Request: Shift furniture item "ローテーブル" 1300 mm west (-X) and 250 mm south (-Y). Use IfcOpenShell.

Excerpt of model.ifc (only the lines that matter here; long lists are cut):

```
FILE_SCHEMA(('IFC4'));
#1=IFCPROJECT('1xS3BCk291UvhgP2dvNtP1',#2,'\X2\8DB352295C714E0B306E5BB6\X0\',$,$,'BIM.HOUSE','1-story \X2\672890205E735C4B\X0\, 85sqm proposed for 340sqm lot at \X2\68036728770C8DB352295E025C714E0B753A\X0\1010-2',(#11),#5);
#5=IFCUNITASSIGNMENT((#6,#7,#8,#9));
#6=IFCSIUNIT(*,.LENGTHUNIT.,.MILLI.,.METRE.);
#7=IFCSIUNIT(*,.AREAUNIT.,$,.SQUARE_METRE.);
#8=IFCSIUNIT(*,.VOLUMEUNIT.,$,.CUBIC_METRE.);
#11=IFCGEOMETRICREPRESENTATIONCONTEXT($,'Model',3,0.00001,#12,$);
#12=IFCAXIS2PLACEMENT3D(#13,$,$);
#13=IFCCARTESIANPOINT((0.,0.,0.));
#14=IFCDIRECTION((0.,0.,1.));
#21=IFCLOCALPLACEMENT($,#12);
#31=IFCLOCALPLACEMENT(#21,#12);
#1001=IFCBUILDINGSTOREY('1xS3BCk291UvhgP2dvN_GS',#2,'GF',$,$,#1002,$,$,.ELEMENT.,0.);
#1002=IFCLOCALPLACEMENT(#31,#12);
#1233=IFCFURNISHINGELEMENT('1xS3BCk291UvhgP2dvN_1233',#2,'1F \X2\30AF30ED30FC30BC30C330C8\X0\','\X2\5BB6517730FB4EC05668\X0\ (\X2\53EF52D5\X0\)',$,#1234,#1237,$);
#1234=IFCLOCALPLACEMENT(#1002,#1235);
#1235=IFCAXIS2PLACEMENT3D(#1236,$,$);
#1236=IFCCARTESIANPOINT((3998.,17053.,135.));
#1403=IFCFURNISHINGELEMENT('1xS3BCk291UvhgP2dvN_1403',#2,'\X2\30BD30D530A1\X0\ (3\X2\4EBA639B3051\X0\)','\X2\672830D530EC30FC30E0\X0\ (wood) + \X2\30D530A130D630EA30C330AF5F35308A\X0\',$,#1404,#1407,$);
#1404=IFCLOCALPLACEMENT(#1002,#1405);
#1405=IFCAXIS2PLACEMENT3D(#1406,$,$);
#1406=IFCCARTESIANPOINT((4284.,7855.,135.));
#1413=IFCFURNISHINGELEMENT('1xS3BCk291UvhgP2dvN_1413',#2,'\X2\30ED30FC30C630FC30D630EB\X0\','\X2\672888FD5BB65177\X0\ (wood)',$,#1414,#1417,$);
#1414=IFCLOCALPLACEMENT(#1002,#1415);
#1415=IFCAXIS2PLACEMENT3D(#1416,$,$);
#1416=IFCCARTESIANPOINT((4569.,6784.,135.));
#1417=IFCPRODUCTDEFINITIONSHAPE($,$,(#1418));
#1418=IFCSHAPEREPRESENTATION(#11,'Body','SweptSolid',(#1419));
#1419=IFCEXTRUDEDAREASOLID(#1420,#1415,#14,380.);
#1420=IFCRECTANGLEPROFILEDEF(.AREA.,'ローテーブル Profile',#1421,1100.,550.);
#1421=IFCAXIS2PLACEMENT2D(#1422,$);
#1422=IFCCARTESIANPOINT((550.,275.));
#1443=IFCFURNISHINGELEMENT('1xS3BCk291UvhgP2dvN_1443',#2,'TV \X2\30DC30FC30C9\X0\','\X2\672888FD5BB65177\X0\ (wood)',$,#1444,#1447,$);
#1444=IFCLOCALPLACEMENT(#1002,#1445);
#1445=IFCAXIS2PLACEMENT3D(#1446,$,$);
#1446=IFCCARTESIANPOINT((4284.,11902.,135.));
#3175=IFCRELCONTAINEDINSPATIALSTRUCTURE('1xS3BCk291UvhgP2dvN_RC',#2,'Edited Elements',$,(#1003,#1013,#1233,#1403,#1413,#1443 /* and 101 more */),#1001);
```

```python
import ifcopenshell
import ifcopenshell.api.geometry
import ifcopenshell.util.placement
import ifcopenshell.util.unit

model = ifcopenshell.open("model.ifc")
unit_scale = ifcopenshell.util.unit.calculate_unit_scale(model)

item = model.by_guid("1xS3BCk291UvhgP2dvN_1413")
matrix = ifcopenshell.util.placement.get_local_placement(item.ObjectPlacement)
matrix[0, 3] -= 1.3 / unit_scale
matrix[1, 3] -= 0.25 / unit_scale
ifcopenshell.api.geometry.edit_object_placement(model, product=item, matrix=matrix, is_si=False)

print(ifcopenshell.util.placement.get_local_placement(item.ObjectPlacement).round(3) + 0.0)

model.write("model_updated.ifc")
```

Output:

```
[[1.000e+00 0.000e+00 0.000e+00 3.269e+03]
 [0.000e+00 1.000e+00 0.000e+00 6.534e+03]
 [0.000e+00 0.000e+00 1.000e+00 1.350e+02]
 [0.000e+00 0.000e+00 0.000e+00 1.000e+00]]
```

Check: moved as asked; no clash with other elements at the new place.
